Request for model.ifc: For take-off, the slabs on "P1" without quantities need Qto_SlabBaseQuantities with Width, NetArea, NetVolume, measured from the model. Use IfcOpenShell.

First a look at what the model holds.

```python
import ifcopenshell
import ifcopenshell.util.element
import ifcopenshell.util.unit

model = ifcopenshell.open("model.ifc")
print(model.schema)
for unit_type in ("LENGTHUNIT", "AREAUNIT", "VOLUMEUNIT"):
    print(unit_type, ifcopenshell.util.unit.calculate_unit_scale(model, unit_type))
storey = next(s for s in model.by_type("IfcBuildingStorey") if s.Name == "P1")
slabs = [e for e in ifcopenshell.util.element.get_decomposition(storey) if e.is_a("IfcSlab")]
for e in sorted(slabs, key=lambda e: e.id()):
    print(e.id(), e.is_a(), e.Name, list(ifcopenshell.util.element.get_psets(e, qtos_only=True)), sep=" | ")
```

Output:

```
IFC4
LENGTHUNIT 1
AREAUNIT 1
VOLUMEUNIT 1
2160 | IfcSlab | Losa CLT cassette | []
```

```python
import ifcopenshell
import ifcopenshell.api.pset
import ifcopenshell.geom
import ifcopenshell.util.element
import ifcopenshell.util.shape
import ifcopenshell.util.unit

model = ifcopenshell.open("model.ifc")
unit_scale = ifcopenshell.util.unit.calculate_unit_scale(model)
area_scale = ifcopenshell.util.unit.calculate_unit_scale(model, "AREAUNIT")
volume_scale = ifcopenshell.util.unit.calculate_unit_scale(model, "VOLUMEUNIT")
settings = ifcopenshell.geom.settings()

storey = next(s for s in model.by_type("IfcBuildingStorey") if s.Name == "P1")
slabs = [e for e in ifcopenshell.util.element.get_decomposition(storey) if e.is_a("IfcSlab")]

for e in sorted(slabs, key=lambda e: e.id()):
    if ifcopenshell.util.element.get_psets(e, qtos_only=True, should_inherit=False):
        continue
    # Geometry comes back in metres, in the element's own axes.
    shape = ifcopenshell.geom.create_shape(settings, e)
    values = {
        "Width": ifcopenshell.util.shape.get_z(shape.geometry) / unit_scale,
        "NetArea": ifcopenshell.util.shape.get_footprint_area(shape.geometry) / area_scale,
        "NetVolume": ifcopenshell.util.shape.get_volume(shape.geometry) / volume_scale,
    }
    qto = ifcopenshell.api.pset.add_qto(model, product=e, name="Qto_SlabBaseQuantities")
    ifcopenshell.api.pset.edit_qto(model, qto=qto, properties=values)
    print(e.id(), {k: round(v, 3) for k, v in values.items()})

model.write("model_edited.ifc")
```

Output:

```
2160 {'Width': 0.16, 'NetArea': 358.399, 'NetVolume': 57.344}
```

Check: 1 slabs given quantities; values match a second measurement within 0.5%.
